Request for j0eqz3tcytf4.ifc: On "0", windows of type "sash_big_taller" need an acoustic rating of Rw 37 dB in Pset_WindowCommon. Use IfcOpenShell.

First a look at what the model holds.

```python
import ifcopenshell
import ifcopenshell.util.element

model = ifcopenshell.open("j0eqz3tcytf4.ifc")
print(model.schema)
storey = next(s for s in model.by_type("IfcBuildingStorey") if s.Name == "0")
windows = [e for e in ifcopenshell.util.element.get_decomposition(storey) if e.is_a("IfcWindow")]
seen = {}
for e in windows:
    element_type = ifcopenshell.util.element.get_type(e)
    key = (element_type.Name if element_type != e and element_type else None, ifcopenshell.util.element.get_pset(e, "Pset_WindowCommon", "AcousticRating"))
    seen[key] = seen.get(key, 0) + 1
for (name, value), count in sorted(seen.items(), key=str):
    print(count, "x", name, "|", value)
```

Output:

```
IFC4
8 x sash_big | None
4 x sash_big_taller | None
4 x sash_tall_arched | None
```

```python
import ifcopenshell
import ifcopenshell.api.pset
import ifcopenshell.util.element

model = ifcopenshell.open("j0eqz3tcytf4.ifc")

storey = next(s for s in model.by_type("IfcBuildingStorey") if s.Name == "0")
windows = [e for e in ifcopenshell.util.element.get_decomposition(storey) if e.is_a("IfcWindow")]

count = 0
for e in windows:
    element_type = ifcopenshell.util.element.get_type(e)
    if element_type in (None, e) or element_type.Name != "sash_big_taller":
        continue
    # add_pset returns the element's existing set when there is one.
    pset = ifcopenshell.api.pset.add_pset(model, product=e, name="Pset_WindowCommon")
    ifcopenshell.api.pset.edit_pset(model, pset=pset, properties={"AcousticRating": "Rw 37 dB"})
    count += 1

print(count, "windows updated")

model.write("j0eqz3tcytf4_v2.ifc")
```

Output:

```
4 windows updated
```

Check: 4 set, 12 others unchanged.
